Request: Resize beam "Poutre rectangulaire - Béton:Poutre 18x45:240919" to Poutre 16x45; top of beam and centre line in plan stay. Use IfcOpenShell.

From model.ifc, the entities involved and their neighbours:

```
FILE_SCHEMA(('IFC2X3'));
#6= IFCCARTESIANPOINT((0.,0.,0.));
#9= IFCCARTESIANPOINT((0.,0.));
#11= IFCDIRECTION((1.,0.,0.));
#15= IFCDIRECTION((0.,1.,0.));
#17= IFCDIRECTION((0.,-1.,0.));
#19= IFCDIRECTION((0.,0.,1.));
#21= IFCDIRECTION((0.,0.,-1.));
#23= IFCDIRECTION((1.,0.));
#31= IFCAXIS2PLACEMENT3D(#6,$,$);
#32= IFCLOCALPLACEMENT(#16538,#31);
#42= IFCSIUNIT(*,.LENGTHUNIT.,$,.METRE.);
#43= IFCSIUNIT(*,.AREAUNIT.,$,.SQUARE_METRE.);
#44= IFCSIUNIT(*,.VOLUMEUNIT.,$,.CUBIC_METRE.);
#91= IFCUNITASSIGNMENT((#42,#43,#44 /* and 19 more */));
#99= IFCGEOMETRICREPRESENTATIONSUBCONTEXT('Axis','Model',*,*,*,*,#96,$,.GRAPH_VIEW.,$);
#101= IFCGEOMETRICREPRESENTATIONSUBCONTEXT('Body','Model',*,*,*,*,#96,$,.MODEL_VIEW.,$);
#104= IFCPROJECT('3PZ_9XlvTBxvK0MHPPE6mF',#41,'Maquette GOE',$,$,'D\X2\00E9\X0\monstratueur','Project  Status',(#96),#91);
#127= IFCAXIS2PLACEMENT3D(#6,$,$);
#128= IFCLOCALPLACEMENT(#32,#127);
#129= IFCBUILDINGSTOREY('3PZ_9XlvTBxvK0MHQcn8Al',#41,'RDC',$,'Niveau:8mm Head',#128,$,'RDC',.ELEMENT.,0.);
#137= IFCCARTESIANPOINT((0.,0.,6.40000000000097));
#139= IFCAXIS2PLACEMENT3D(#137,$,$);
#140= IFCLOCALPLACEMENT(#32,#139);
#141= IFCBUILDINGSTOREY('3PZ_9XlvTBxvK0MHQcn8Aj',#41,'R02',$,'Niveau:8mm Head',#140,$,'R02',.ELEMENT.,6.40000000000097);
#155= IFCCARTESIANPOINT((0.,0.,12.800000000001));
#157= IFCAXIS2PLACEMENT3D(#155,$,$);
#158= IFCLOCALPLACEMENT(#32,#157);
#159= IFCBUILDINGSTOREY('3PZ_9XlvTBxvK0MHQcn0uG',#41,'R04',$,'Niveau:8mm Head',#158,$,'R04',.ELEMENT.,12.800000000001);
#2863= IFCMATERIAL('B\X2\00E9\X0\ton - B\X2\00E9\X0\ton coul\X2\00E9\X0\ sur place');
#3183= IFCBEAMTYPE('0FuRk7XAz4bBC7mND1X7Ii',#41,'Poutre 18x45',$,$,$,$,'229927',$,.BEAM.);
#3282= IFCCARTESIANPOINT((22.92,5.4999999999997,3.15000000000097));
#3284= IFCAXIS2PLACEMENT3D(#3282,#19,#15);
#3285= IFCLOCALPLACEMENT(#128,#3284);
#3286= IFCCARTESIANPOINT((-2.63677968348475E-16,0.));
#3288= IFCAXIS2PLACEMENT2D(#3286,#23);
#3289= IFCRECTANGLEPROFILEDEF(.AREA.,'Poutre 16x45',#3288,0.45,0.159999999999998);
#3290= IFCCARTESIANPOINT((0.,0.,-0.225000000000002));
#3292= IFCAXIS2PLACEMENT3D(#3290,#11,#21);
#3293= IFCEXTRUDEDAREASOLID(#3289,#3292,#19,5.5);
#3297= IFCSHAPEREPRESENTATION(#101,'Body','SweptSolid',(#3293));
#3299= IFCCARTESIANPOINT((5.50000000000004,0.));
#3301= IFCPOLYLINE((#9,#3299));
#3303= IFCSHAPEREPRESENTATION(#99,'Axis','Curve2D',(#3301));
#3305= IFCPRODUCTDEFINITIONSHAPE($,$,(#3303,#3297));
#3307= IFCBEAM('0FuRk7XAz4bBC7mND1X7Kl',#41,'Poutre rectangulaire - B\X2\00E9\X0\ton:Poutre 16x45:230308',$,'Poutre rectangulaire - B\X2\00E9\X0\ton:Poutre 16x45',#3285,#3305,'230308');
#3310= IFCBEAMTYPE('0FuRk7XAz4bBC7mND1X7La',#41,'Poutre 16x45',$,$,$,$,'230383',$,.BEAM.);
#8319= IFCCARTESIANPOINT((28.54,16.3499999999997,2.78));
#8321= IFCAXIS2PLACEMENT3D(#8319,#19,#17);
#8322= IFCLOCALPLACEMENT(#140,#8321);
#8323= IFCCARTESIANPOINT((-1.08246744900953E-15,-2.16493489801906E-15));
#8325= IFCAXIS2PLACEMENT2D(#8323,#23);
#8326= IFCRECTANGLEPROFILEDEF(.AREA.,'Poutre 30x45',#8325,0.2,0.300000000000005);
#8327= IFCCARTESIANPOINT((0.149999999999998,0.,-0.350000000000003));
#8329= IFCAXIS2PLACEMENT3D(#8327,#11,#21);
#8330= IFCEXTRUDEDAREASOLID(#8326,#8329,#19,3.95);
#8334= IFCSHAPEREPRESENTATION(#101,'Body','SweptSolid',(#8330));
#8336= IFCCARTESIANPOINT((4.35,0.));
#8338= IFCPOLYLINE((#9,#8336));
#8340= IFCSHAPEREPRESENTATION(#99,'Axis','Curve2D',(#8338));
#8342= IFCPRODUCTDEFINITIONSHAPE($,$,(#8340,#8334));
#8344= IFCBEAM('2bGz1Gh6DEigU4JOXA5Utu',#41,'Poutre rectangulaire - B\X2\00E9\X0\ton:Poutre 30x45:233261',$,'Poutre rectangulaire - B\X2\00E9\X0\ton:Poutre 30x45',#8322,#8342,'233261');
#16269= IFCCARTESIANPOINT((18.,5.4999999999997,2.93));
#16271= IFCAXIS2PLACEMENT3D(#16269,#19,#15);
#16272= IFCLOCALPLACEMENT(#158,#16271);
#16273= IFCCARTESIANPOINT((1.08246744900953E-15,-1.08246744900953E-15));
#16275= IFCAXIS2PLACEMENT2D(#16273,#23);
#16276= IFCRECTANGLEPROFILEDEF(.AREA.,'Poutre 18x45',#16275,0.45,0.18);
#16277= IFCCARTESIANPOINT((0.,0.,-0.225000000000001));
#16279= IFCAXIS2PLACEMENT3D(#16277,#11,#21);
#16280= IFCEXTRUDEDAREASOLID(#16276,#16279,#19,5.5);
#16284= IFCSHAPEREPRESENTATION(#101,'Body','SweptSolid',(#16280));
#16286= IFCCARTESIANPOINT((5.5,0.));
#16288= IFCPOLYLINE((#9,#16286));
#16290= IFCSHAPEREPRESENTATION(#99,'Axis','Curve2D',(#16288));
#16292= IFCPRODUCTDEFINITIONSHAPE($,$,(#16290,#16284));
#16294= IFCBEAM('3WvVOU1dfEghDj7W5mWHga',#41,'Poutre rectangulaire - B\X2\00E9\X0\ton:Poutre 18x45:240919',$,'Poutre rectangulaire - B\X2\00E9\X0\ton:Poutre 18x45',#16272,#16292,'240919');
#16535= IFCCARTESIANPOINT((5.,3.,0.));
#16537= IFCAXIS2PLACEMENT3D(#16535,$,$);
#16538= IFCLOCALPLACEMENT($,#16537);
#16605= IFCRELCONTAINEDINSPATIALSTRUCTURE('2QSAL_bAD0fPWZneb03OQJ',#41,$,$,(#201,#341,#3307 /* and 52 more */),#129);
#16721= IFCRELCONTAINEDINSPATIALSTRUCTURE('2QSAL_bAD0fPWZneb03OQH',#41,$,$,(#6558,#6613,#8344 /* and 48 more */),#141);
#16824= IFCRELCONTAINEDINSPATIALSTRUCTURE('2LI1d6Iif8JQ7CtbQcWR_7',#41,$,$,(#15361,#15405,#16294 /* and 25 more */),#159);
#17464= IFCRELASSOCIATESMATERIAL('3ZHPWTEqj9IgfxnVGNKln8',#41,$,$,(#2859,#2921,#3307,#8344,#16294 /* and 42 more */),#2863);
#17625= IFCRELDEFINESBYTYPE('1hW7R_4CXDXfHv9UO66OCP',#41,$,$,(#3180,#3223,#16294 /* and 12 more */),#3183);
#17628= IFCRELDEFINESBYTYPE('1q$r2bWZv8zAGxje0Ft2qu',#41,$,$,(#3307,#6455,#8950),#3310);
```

```python
import ifcopenshell
import ifcopenshell.api.type
import ifcopenshell.util.element
import ifcopenshell.util.representation

model = ifcopenshell.open("model.ifc")

member = model.by_id(16294)
source = next(p for p in model.by_type("IfcRectangleProfileDef") if p.ProfileName == "Poutre 16x45")

body = ifcopenshell.util.representation.get_representation(member, "Model", "Body")
solid = body.Items[0]
old_profile = solid.SweptArea

# Copy the section's sizes but keep this member's own profile position.
profile = ifcopenshell.util.element.copy(model, source)
# Profiles are centred, so shift by half the change in depth to hold the top.
shift = (old_profile.XDim - profile.XDim) / 2
x, y = old_profile.Position.Location.Coordinates
up = (-1.0, 0.0)  # upwards, in the solid's own plane
location = model.createIfcCartesianPoint((x + up[0] * shift, y + up[1] * shift))
profile.Position = model.createIfcAxis2Placement2D(location, old_profile.Position.RefDirection)
solid.SweptArea = profile
if not model.get_total_inverses(old_profile):
    ifcopenshell.util.element.remove_deep2(model, old_profile)

new_type = model.by_guid("0FuRk7XAz4bBC7mND1X7La")
ifcopenshell.api.type.assign_type(
    model, related_objects=[member], relating_type=new_type, should_map_representations=False
)
member.Name = member.Name.replace("Poutre 18x45", "Poutre 16x45")
member.ObjectType = "Poutre rectangulaire - Béton:Poutre 16x45"

print(solid.SweptArea)

model.write("model_edited.ifc")
```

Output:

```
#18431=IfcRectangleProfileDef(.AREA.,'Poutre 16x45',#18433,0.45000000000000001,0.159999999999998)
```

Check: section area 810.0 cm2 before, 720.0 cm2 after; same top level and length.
